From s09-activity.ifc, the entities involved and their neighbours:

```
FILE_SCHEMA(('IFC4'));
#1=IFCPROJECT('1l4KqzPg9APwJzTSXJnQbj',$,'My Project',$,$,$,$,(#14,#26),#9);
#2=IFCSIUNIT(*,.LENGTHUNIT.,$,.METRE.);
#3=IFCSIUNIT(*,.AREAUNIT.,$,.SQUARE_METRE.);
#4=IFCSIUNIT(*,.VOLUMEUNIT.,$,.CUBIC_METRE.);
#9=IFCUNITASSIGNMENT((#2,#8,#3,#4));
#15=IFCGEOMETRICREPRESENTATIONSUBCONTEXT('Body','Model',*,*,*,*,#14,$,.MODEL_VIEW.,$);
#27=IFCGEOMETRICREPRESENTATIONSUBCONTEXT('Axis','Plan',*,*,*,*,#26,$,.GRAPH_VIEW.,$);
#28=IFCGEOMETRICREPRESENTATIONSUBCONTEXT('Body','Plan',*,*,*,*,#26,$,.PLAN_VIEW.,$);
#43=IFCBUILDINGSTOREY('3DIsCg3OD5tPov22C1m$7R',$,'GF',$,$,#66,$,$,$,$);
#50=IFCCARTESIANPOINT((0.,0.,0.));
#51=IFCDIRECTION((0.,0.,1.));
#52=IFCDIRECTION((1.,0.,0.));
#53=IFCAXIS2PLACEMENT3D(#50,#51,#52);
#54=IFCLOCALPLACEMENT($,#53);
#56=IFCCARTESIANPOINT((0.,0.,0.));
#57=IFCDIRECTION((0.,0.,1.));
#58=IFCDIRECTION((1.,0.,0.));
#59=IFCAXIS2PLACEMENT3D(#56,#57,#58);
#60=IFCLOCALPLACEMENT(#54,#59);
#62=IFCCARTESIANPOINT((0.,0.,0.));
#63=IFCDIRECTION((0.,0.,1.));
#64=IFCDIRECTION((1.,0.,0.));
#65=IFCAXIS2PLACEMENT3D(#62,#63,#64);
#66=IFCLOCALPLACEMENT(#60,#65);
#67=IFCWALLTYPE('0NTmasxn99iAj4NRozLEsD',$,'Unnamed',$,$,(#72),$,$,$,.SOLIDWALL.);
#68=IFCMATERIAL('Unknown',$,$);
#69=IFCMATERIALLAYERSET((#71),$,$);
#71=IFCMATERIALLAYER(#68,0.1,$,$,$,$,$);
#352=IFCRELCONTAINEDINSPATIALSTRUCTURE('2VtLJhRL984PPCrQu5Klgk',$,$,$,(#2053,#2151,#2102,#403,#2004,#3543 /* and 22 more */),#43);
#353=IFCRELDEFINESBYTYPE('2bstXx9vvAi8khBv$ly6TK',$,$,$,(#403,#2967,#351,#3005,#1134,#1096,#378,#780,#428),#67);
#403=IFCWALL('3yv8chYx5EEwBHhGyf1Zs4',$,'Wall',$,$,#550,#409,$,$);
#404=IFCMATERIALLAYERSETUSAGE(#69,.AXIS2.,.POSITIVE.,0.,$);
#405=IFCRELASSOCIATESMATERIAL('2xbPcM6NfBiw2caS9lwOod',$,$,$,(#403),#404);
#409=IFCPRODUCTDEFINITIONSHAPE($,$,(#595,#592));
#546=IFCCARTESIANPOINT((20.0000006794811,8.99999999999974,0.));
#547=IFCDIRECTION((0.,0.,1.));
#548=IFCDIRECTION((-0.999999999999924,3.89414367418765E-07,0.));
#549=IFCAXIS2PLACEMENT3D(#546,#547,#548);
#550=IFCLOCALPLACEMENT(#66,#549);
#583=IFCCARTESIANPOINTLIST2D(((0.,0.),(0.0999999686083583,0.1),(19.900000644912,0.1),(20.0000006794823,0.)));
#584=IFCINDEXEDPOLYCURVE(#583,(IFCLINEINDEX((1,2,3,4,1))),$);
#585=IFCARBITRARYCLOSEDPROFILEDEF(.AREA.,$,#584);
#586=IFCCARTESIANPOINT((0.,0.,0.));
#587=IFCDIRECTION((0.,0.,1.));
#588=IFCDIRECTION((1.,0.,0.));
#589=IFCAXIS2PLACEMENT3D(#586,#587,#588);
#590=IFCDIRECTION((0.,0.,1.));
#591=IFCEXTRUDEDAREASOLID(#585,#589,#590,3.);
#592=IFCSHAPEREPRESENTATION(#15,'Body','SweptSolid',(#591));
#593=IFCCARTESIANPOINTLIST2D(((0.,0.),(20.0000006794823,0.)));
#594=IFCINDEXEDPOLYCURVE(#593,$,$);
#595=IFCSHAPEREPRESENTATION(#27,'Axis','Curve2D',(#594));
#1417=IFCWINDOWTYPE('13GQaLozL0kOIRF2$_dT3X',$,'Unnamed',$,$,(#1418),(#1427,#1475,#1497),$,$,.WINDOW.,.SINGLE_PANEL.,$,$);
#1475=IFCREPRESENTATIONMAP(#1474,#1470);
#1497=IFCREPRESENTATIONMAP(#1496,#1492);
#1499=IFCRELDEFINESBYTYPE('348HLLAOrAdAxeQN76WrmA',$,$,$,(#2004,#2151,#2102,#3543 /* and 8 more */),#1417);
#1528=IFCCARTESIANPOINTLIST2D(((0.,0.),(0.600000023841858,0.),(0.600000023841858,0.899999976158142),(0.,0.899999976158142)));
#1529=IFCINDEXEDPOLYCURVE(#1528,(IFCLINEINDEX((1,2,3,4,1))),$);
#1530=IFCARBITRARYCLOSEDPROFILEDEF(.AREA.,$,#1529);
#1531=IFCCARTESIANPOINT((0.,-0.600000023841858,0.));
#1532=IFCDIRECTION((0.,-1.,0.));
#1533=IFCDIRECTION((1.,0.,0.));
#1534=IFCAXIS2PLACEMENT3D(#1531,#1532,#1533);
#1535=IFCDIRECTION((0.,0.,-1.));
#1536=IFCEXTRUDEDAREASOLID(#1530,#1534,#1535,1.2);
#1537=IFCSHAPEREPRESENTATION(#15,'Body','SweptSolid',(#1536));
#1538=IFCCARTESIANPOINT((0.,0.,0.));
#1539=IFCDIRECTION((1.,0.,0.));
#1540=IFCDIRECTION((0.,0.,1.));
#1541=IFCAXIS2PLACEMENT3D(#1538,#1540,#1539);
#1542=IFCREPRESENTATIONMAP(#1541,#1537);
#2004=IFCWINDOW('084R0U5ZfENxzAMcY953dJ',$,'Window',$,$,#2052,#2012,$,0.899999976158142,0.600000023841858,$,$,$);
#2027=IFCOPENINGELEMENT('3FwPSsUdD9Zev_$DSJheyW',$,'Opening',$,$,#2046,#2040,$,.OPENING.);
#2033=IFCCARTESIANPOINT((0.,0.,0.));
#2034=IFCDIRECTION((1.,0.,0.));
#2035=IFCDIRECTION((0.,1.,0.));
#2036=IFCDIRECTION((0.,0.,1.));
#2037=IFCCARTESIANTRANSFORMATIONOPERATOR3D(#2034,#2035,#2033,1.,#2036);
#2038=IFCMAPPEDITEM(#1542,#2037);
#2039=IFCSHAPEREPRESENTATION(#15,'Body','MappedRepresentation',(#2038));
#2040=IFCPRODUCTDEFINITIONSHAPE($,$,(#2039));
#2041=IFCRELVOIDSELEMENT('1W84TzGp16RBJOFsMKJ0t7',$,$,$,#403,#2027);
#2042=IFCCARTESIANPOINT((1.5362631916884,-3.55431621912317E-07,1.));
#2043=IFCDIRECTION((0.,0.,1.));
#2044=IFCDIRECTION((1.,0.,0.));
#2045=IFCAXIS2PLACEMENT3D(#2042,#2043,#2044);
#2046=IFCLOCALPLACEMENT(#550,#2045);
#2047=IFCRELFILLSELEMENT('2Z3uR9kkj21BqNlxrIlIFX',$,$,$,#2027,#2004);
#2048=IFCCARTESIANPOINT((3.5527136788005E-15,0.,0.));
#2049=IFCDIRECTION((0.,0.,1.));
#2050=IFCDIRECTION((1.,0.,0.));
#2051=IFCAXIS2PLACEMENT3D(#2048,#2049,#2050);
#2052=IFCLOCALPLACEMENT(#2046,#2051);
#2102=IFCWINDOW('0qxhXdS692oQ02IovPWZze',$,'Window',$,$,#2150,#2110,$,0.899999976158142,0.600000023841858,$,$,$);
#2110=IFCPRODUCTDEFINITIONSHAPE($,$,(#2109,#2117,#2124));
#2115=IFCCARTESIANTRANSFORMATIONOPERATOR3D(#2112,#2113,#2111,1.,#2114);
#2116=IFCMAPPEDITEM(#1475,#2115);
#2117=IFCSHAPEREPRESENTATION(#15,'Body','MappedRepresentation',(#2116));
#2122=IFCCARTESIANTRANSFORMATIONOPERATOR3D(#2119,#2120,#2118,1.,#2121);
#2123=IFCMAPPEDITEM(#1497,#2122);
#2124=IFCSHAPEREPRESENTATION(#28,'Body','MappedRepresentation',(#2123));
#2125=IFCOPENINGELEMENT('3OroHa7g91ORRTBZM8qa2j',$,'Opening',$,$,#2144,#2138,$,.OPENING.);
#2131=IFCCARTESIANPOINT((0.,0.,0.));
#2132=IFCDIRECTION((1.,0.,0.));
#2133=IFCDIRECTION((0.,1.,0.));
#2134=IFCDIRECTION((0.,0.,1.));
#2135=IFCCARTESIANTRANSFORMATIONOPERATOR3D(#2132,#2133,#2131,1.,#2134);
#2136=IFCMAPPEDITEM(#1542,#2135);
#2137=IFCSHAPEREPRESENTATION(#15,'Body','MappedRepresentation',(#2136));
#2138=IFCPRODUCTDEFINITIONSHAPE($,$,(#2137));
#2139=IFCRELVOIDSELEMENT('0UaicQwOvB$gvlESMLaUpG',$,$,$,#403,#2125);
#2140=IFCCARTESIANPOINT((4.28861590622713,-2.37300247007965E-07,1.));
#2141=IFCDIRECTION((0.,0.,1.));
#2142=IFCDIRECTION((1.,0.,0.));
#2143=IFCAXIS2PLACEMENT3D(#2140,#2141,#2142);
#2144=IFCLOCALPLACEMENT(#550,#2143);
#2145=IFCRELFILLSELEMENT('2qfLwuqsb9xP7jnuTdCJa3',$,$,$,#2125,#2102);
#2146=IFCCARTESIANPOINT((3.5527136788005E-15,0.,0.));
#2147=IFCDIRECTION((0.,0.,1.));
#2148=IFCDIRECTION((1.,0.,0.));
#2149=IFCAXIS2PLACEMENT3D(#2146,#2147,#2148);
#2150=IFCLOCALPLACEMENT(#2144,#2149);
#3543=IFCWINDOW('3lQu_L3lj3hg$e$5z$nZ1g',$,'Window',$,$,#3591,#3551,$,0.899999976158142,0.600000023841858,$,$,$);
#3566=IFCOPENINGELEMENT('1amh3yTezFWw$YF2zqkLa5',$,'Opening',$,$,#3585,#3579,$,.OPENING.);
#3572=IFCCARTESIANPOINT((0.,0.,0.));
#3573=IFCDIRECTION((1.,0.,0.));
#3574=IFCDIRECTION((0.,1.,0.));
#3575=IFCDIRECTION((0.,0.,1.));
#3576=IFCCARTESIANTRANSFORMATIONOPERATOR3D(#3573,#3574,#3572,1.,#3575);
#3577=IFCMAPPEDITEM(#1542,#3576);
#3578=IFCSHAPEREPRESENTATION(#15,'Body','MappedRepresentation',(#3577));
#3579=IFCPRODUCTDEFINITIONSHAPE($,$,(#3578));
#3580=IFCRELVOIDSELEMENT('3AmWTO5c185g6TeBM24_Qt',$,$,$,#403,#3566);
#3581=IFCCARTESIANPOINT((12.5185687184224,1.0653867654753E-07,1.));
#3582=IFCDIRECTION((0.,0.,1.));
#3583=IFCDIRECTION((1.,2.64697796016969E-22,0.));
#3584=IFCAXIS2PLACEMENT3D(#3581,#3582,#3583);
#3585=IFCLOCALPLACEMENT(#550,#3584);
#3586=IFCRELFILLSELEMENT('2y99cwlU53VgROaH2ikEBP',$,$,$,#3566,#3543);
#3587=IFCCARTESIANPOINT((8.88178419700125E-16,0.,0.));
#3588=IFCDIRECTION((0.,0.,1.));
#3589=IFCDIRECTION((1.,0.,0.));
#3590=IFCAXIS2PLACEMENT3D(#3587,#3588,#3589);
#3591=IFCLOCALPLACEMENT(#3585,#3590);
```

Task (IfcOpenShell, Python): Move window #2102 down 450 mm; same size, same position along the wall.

```python
import numpy as np
import ifcopenshell
import ifcopenshell.api.geometry
import ifcopenshell.util.placement
import ifcopenshell.util.unit

model = ifcopenshell.open("s09-activity.ifc")
unit_scale = ifcopenshell.util.unit.calculate_unit_scale(model)

window = model.by_guid("0qxhXdS692oQ02IovPWZze")
opening = window.FillsVoids[0].RelatingOpeningElement
dz = -0.45

shift = np.array([0.0, 0.0, dz])
# The window is placed relative to its opening, so it follows when the opening moves.
matrix = ifcopenshell.util.placement.get_local_placement(opening.ObjectPlacement)
matrix[:3, 3] += shift
ifcopenshell.api.geometry.edit_object_placement(
    model, product=opening, matrix=matrix, is_si=False, should_transform_children=True
)

print(f"moved by {dz * unit_scale:+.3f} m")

model.write("s09-activity-out.ifc")
```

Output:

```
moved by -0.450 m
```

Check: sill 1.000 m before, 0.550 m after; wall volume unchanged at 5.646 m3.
